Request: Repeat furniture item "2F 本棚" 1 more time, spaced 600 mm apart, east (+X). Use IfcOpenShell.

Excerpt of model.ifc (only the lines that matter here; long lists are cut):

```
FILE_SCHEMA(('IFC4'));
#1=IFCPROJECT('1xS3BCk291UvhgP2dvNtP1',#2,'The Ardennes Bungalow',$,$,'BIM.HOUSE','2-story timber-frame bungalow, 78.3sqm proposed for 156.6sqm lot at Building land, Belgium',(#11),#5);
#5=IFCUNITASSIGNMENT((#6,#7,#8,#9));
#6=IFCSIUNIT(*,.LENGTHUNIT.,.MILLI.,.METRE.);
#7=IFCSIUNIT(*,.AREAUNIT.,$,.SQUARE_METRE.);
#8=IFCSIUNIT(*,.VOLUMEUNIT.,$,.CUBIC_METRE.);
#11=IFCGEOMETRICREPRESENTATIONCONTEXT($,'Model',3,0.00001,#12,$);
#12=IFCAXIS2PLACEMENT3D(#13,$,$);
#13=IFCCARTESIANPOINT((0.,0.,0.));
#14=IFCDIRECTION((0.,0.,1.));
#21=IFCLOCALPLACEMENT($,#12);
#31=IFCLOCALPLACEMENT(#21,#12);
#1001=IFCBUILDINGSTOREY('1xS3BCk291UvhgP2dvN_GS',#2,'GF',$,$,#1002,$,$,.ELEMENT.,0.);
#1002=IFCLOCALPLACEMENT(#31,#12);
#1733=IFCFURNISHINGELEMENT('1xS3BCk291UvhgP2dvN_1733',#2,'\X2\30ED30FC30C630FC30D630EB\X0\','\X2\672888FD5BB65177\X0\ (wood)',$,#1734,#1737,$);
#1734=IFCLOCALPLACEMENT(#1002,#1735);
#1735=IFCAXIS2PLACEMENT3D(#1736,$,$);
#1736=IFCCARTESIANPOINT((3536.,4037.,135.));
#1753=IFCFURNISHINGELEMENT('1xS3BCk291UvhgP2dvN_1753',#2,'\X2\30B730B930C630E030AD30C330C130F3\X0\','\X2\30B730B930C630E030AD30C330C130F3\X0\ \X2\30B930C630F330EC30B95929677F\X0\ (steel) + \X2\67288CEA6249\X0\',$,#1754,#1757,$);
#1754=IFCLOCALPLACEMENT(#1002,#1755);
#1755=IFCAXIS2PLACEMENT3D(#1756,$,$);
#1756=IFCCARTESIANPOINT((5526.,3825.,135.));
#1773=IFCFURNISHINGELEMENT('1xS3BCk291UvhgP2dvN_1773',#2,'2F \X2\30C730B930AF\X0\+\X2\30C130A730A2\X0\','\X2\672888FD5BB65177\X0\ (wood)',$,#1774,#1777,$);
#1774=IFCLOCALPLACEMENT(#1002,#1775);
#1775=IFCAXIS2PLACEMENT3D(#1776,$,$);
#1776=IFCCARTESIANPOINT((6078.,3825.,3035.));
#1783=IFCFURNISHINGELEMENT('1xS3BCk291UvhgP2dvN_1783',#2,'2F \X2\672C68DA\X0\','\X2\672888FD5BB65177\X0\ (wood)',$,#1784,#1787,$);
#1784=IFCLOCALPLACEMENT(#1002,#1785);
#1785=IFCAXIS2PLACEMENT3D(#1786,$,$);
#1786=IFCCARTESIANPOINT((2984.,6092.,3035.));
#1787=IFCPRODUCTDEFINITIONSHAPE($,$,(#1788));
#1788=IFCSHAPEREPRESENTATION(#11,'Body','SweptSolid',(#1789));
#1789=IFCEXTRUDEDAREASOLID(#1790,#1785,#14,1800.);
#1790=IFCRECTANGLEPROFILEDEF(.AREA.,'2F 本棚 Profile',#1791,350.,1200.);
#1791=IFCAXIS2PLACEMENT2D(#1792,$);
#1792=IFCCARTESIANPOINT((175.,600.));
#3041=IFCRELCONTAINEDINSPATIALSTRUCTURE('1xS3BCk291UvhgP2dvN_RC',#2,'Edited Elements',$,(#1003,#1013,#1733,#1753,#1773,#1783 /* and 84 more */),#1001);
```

```python
import numpy as np
import ifcopenshell
import ifcopenshell.api.geometry
import ifcopenshell.api.root
import ifcopenshell.util.element
import ifcopenshell.util.placement
import ifcopenshell.util.unit

model = ifcopenshell.open("model.ifc")
unit_scale = ifcopenshell.util.unit.calculate_unit_scale(model)


def reuse_history(source, copy):
    """copy_class also copies each property set's owner history, people and application; keep the originals."""
    for rel in copy.IsDefinedBy:
        if rel.is_a("IfcRelDefinesByProperties") and (history := rel.RelatingPropertyDefinition.OwnerHistory):
            rel.RelatingPropertyDefinition.OwnerHistory = source.OwnerHistory
            ifcopenshell.util.element.remove_deep2(model, history)


source = model.by_id(1783)
base = ifcopenshell.util.placement.get_local_placement(source.ObjectPlacement)
step = np.array([1.0, 0.0, 0.0]) * 0.6 / unit_scale

for i in range(1, 2):
    copy = ifcopenshell.api.root.copy_class(model, product=source)
    copy.Representation = ifcopenshell.util.element.copy_deep(
        model, source.Representation, exclude=["IfcGeometricRepresentationContext", "IfcRepresentationMap"]
    )
    reuse_history(source, copy)
    matrix = base.copy()
    matrix[:3, 3] += i * step
    print("added at", matrix[:3, 3].round(3) + 0.0)
    ifcopenshell.api.geometry.edit_object_placement(model, product=copy, matrix=matrix, is_si=False)

model.write("model_v2.ifc")
```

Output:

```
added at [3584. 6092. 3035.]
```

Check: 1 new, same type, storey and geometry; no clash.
